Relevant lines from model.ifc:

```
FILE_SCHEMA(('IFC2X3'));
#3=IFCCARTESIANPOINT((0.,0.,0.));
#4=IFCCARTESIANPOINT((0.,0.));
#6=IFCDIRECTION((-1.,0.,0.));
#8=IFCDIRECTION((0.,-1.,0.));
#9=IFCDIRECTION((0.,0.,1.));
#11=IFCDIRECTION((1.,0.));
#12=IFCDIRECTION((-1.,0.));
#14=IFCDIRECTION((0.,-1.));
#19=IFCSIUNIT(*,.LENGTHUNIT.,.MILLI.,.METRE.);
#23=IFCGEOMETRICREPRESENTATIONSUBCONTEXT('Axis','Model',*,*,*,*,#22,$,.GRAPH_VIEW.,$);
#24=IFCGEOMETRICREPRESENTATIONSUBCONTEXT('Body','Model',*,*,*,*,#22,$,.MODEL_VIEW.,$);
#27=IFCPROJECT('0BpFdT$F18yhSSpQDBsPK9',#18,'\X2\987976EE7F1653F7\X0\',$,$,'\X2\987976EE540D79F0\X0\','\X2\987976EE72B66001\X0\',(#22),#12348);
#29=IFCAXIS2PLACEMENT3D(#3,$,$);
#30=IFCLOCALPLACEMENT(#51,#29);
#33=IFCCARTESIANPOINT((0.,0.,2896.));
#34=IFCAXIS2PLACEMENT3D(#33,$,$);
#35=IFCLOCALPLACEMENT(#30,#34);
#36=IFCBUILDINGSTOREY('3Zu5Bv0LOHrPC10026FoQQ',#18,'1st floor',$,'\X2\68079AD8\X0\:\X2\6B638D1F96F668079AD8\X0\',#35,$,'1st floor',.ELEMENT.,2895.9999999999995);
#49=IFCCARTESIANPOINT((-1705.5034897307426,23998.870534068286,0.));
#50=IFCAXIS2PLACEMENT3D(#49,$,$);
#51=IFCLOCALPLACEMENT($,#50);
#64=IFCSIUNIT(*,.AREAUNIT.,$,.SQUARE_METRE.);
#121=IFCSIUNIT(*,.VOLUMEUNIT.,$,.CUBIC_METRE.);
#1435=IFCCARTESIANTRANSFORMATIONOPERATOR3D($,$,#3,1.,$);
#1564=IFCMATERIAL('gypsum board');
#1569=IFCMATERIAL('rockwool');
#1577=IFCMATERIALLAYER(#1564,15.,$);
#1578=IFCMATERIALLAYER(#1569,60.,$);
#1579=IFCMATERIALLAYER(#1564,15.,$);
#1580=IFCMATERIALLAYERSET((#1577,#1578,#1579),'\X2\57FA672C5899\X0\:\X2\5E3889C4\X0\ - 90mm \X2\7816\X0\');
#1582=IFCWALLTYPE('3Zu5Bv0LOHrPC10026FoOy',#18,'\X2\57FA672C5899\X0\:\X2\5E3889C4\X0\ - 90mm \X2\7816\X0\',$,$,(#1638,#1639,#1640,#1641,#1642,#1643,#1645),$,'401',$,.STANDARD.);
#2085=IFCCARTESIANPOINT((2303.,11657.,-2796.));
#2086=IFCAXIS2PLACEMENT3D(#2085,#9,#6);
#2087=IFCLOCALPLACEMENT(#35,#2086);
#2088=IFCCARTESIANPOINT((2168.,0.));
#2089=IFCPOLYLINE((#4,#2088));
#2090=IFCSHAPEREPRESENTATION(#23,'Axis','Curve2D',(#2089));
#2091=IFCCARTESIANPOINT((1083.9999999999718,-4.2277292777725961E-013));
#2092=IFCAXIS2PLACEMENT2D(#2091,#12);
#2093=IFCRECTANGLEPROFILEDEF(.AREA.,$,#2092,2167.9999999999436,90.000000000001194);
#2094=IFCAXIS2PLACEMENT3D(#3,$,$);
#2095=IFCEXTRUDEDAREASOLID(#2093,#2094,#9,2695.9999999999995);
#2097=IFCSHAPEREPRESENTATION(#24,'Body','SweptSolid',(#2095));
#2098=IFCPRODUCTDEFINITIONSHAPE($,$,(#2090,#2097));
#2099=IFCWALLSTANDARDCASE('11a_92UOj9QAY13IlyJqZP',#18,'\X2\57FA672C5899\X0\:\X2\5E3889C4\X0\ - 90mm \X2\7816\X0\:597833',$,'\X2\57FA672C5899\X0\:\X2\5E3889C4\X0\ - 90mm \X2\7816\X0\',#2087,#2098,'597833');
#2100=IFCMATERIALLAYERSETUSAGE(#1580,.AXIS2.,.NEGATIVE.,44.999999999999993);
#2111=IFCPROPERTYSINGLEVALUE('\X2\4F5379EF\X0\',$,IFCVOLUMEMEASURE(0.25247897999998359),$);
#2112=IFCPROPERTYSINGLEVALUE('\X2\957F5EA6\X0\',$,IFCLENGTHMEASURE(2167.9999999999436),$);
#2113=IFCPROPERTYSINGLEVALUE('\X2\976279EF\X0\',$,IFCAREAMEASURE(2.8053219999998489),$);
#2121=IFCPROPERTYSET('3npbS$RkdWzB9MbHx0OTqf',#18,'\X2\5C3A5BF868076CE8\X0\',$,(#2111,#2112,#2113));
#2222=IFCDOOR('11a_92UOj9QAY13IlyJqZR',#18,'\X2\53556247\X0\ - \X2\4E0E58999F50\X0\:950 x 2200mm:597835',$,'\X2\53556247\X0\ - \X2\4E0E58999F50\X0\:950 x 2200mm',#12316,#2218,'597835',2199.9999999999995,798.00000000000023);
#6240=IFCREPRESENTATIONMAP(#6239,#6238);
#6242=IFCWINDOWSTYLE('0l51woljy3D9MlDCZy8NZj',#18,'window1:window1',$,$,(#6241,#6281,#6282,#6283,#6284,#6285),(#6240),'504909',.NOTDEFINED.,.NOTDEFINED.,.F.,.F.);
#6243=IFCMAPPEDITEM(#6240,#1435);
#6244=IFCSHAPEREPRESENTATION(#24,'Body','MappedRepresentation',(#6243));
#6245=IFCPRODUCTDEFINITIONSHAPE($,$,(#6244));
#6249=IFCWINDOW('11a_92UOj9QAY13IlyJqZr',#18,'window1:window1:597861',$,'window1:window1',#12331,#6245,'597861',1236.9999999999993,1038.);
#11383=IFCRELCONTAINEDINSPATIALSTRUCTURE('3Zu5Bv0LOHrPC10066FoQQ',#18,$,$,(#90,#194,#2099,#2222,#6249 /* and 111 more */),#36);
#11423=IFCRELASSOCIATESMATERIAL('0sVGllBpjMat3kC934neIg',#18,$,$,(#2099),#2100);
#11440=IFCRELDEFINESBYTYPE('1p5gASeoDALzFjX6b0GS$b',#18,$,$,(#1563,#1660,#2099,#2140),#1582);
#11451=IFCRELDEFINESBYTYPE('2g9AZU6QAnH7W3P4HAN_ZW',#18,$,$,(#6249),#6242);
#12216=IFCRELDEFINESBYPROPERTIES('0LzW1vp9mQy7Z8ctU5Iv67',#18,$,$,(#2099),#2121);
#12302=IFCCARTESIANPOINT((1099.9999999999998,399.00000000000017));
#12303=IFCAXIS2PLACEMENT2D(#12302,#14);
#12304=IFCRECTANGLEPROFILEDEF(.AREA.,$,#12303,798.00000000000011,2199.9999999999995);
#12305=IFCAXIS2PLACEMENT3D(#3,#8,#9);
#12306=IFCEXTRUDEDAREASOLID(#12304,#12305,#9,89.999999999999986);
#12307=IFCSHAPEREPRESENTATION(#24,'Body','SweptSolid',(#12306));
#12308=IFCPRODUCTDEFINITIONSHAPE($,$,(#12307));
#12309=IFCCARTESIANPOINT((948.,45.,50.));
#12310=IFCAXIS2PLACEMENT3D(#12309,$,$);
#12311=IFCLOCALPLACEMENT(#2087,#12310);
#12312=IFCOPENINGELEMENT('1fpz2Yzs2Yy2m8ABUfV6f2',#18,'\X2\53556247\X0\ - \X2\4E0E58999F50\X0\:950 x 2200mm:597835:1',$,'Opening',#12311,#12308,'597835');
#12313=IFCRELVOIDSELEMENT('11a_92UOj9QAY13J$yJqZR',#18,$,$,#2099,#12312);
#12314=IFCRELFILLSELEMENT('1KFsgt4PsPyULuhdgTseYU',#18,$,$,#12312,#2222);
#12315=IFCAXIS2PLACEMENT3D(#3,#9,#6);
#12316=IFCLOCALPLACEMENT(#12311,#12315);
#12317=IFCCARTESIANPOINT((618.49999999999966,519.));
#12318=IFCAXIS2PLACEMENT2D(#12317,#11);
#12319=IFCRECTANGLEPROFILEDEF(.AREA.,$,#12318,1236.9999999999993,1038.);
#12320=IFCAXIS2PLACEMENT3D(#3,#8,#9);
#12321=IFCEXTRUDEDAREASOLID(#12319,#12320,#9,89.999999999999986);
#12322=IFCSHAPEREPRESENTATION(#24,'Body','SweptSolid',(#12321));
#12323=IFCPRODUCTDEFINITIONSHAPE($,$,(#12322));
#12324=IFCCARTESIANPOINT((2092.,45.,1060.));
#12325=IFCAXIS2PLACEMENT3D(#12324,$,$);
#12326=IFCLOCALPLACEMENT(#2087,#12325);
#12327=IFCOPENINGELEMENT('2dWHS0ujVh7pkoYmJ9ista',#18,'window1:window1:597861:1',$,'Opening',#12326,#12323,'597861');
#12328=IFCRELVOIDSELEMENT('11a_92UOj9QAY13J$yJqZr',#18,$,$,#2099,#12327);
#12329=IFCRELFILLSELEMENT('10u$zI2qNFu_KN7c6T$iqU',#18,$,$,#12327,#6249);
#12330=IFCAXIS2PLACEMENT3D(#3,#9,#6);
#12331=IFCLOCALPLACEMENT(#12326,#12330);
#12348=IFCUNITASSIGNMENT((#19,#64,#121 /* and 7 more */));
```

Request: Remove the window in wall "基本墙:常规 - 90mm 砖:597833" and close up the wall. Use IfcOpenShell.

```python
import ifcopenshell
import ifcopenshell.api.feature
import ifcopenshell.api.pset
import ifcopenshell.api.root
import ifcopenshell.geom
import ifcopenshell.util.element
import ifcopenshell.util.shape
import ifcopenshell.util.unit

model = ifcopenshell.open("model.ifc")
area_scale = ifcopenshell.util.unit.calculate_unit_scale(model, "AREAUNIT")
volume_scale = ifcopenshell.util.unit.calculate_unit_scale(model, "VOLUMEUNIT")
settings = ifcopenshell.geom.settings()


def volume(element):
    """Net volume in cubic metres, openings subtracted."""
    shape = ifcopenshell.geom.create_shape(settings, element)
    return ifcopenshell.util.shape.get_volume(shape.geometry)


window = model.by_guid("11a_92UOj9QAY13IlyJqZr")
opening = window.FillsVoids[0].RelatingOpeningElement
wall = opening.VoidsElements[0].RelatingBuildingElement
before = volume(wall)

ifcopenshell.api.root.remove_product(model, product=window)
ifcopenshell.api.feature.remove_feature(model, feature=opening)

after = volume(wall)
thickness = 0.09  # wall thickness in metres

# Update the wall's stored quantities.
pset = model.by_id(ifcopenshell.util.element.get_pset(wall, "尺寸标注", should_inherit=False)["id"])
ifcopenshell.api.pset.edit_pset(model, pset=pset, properties={
    "体积": model.create_entity("IfcVolumeMeasure", after / volume_scale),
    "面积": model.create_entity("IfcAreaMeasure", after / thickness / area_scale),
})

print(f"wall volume {before:.3f} -> {after:.3f} m3")

model.write("model-out.ifc")
```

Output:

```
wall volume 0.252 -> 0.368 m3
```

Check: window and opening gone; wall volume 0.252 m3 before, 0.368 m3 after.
